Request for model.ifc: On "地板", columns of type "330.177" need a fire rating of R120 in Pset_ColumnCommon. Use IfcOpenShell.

First a look at what the model holds.

```python
import ifcopenshell
import ifcopenshell.util.element

model = ifcopenshell.open("model.ifc")
print(model.schema)
storey = next(s for s in model.by_type("IfcBuildingStorey") if s.Name == "地板")
columns = [e for e in ifcopenshell.util.element.get_decomposition(storey) if e.is_a("IfcColumn")]
seen = {}
for e in columns:
    element_type = ifcopenshell.util.element.get_type(e)
    key = (element_type.Name if element_type != e and element_type else None, ifcopenshell.util.element.get_pset(e, "Pset_ColumnCommon", "FireRating"))
    seen[key] = seen.get(key, 0) + 1
for (name, value), count in sorted(seen.items(), key=str):
    print(count, "x", name, "|", value)
```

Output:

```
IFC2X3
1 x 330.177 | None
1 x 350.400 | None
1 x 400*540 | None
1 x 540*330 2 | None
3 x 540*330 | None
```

```python
import ifcopenshell
import ifcopenshell.api.pset
import ifcopenshell.util.element

model = ifcopenshell.open("model.ifc")

storey = next(s for s in model.by_type("IfcBuildingStorey") if s.Name == "地板")
columns = [e for e in ifcopenshell.util.element.get_decomposition(storey) if e.is_a("IfcColumn")]

count = 0
for e in columns:
    element_type = ifcopenshell.util.element.get_type(e)
    if element_type in (None, e) or element_type.Name != "330.177":
        continue
    # add_pset returns the element's existing set when there is one.
    pset = ifcopenshell.api.pset.add_pset(model, product=e, name="Pset_ColumnCommon")
    ifcopenshell.api.pset.edit_pset(model, pset=pset, properties={"FireRating": "R120"})
    count += 1

print(count, "columns updated")

model.write("model_rev.ifc")
```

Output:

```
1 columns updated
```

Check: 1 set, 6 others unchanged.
